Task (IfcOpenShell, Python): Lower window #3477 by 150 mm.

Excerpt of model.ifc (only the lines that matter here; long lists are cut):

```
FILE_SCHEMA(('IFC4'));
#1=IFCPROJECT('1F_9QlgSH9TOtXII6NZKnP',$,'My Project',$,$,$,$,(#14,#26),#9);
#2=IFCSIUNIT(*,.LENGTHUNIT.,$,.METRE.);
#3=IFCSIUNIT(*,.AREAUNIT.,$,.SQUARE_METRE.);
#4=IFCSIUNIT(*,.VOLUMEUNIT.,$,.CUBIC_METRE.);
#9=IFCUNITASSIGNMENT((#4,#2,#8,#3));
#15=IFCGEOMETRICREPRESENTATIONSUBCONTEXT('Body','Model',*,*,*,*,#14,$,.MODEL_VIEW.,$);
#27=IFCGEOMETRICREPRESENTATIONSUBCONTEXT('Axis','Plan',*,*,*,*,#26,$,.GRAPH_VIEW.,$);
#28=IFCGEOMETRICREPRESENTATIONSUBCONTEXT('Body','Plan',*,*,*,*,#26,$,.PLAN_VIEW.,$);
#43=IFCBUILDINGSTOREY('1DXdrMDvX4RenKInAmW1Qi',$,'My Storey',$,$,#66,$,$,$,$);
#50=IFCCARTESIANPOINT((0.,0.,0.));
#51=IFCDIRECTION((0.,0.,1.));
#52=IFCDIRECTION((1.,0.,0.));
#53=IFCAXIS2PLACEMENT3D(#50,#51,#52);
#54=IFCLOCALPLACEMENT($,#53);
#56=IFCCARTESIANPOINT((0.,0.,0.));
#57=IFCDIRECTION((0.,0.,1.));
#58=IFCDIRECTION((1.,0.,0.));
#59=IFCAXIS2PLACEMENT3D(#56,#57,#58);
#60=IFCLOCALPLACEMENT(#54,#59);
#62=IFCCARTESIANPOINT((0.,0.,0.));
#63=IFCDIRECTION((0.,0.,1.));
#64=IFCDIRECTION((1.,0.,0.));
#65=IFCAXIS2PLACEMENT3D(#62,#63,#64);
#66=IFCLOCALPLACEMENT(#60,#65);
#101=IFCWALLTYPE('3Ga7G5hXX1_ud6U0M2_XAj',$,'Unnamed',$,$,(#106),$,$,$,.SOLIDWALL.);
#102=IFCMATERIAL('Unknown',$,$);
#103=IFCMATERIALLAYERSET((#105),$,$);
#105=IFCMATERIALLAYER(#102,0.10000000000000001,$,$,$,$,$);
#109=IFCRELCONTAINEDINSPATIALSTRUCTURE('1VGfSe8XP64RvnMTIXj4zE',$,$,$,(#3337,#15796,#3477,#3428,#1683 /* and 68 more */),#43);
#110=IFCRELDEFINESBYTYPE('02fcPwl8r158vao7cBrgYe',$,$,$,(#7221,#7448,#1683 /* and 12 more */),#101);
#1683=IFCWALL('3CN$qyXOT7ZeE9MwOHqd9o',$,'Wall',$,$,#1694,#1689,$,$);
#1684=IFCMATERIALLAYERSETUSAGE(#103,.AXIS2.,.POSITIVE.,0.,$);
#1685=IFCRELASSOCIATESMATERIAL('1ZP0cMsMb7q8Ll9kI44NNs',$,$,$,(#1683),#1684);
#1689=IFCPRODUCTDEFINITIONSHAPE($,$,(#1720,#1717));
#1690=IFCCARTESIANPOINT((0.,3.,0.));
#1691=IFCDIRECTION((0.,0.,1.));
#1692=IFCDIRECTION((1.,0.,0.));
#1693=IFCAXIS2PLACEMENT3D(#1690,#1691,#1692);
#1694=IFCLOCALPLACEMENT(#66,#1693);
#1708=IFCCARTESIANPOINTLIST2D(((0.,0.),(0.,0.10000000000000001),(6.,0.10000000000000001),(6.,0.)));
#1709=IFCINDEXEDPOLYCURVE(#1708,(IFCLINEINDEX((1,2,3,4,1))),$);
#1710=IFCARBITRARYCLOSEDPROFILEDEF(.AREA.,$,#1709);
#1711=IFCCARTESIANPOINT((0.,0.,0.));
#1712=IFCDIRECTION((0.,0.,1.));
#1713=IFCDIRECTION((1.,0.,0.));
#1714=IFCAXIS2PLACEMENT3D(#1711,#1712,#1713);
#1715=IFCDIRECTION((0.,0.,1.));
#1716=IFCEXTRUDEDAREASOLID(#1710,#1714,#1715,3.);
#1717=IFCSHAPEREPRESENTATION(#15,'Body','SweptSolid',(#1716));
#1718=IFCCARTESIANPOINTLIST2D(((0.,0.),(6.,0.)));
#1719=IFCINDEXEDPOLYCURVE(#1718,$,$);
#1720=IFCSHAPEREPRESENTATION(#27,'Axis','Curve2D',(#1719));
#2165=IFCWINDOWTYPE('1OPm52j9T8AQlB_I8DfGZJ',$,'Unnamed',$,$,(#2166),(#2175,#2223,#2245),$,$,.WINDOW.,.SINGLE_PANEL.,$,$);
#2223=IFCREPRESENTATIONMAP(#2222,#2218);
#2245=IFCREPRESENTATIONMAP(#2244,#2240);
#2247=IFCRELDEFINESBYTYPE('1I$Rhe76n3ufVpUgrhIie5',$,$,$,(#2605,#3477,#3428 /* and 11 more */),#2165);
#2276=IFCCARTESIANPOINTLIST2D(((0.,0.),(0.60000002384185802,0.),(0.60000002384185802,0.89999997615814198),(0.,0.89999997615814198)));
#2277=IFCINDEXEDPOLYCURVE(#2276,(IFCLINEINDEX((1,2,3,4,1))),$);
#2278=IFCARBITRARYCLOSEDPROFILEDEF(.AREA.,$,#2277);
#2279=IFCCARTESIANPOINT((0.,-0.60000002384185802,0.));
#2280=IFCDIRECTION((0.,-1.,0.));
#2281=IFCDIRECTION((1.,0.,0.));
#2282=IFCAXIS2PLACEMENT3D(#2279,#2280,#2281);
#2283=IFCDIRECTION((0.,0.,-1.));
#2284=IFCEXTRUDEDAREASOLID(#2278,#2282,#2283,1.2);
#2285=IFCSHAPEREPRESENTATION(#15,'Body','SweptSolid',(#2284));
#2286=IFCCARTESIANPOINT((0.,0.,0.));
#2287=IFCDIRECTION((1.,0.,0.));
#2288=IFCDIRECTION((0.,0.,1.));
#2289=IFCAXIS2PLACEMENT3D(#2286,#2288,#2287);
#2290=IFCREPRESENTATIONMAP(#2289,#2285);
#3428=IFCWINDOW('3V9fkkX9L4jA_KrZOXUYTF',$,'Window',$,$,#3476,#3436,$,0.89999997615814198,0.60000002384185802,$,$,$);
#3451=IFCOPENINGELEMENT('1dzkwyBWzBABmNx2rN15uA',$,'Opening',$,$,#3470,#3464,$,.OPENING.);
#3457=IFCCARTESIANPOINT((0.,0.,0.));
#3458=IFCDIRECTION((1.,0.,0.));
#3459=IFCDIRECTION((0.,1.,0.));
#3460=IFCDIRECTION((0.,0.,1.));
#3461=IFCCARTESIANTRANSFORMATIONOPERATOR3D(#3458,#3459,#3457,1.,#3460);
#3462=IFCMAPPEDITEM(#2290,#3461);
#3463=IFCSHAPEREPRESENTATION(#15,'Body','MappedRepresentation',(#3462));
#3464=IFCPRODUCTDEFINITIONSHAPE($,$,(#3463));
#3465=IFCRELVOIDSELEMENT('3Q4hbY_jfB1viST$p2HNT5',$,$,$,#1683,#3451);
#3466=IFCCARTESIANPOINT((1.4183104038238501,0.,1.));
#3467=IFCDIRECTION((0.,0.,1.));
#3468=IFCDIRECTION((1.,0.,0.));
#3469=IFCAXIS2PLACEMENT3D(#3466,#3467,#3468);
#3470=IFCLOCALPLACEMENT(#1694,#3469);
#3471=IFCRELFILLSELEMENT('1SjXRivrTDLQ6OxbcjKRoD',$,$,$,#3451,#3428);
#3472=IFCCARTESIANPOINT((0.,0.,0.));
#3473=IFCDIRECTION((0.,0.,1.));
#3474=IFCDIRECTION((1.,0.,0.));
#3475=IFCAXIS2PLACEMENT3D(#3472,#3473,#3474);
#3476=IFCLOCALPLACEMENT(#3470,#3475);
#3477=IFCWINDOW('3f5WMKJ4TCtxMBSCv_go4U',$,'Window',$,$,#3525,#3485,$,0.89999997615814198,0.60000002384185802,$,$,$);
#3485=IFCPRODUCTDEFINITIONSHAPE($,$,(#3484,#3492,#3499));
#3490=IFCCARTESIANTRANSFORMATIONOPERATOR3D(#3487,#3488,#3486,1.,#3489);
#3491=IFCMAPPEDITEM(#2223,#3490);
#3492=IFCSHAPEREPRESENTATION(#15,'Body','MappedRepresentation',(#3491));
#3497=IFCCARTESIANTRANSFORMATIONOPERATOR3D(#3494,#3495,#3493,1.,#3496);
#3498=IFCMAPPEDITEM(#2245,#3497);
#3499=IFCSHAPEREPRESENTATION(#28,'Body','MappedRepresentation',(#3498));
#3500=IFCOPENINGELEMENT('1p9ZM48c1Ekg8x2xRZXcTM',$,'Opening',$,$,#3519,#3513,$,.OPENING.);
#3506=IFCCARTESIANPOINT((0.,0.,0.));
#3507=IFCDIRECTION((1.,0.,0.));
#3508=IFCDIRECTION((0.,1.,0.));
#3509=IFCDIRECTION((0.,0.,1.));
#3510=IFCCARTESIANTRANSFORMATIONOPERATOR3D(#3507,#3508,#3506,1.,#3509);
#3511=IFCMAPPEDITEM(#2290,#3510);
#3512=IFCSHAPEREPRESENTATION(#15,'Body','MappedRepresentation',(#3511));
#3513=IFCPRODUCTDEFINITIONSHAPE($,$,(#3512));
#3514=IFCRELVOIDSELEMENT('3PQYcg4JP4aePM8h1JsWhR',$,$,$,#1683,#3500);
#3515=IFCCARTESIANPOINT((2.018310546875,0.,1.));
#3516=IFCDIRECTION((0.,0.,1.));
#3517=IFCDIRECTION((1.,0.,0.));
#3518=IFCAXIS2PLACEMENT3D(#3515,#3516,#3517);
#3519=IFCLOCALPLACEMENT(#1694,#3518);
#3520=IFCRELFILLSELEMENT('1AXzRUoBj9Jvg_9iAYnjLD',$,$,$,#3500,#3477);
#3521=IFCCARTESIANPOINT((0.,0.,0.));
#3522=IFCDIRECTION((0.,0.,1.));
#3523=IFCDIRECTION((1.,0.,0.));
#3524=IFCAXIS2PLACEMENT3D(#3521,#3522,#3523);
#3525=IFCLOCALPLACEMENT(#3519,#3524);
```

```python
import numpy as np
import ifcopenshell
import ifcopenshell.api.geometry
import ifcopenshell.util.placement
import ifcopenshell.util.unit

model = ifcopenshell.open("model.ifc")
unit_scale = ifcopenshell.util.unit.calculate_unit_scale(model)

window = model.by_id(3477)
opening = window.FillsVoids[0].RelatingOpeningElement
dz = -0.15 / unit_scale

shift = np.array([0.0, 0.0, dz])
# The window is placed relative to its opening, so it follows when the opening moves.
matrix = ifcopenshell.util.placement.get_local_placement(opening.ObjectPlacement)
matrix[:3, 3] += shift
ifcopenshell.api.geometry.edit_object_placement(
    model, product=opening, matrix=matrix, is_si=False, should_transform_children=True
)

print(f"moved by {dz * unit_scale:+.3f} m")

model.write("model_rev.ifc")
```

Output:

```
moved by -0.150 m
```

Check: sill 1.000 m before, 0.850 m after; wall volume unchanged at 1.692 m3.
